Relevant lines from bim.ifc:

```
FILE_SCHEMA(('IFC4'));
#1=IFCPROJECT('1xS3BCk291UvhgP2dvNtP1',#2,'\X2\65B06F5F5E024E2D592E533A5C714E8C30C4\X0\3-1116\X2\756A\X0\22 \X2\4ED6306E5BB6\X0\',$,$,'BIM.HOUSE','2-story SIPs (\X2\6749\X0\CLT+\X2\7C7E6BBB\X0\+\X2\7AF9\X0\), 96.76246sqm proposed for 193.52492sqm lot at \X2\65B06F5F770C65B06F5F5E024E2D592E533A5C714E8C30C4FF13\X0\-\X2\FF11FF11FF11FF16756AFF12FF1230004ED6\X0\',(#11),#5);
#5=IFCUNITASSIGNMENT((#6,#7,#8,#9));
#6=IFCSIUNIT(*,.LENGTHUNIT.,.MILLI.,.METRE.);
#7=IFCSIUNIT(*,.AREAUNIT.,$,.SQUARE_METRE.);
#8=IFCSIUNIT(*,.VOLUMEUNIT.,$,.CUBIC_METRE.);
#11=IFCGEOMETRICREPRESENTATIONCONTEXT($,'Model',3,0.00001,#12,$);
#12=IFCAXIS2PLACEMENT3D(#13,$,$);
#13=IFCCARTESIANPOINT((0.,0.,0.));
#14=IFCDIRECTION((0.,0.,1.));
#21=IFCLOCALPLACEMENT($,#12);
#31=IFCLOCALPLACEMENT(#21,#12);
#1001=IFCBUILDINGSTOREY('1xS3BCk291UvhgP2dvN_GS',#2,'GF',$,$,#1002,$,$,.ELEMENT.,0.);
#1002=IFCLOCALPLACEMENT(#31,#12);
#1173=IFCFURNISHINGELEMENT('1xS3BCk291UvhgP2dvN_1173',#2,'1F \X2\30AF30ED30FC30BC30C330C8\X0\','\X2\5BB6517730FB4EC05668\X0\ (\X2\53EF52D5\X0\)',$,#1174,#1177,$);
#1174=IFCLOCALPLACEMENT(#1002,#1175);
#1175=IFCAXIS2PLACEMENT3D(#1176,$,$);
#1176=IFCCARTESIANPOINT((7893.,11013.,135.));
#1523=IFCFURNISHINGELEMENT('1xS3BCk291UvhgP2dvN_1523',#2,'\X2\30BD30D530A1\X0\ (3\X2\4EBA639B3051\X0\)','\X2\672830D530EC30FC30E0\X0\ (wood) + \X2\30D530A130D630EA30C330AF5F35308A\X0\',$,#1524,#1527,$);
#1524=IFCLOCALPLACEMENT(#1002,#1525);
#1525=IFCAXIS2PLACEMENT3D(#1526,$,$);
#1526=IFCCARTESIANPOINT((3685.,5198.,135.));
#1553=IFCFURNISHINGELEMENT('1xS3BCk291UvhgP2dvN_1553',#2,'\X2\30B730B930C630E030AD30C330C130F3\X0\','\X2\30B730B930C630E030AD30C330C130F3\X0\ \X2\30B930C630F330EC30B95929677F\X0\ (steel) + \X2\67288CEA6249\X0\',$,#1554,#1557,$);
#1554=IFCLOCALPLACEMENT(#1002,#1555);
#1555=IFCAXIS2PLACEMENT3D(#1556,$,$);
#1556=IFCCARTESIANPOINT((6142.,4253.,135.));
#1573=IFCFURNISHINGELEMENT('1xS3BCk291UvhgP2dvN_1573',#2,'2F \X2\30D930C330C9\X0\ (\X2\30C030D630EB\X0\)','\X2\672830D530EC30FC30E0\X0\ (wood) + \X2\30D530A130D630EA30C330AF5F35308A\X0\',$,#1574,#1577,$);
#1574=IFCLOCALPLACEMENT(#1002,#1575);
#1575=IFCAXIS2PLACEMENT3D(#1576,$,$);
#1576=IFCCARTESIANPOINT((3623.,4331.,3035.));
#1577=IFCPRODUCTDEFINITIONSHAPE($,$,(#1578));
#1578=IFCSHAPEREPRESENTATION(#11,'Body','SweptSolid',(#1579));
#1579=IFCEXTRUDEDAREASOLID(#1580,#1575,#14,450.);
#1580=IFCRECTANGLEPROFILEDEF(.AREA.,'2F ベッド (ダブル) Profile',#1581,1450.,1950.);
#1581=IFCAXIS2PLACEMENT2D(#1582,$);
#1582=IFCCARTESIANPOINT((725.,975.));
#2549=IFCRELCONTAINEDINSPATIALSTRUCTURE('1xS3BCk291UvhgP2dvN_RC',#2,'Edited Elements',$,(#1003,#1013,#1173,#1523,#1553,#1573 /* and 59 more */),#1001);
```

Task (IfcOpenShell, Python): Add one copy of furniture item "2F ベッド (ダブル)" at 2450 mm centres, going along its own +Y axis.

```python
import ifcopenshell
import ifcopenshell.api.geometry
import ifcopenshell.api.root
import ifcopenshell.util.element
import ifcopenshell.util.placement

model = ifcopenshell.open("bim.ifc")


def reuse_history(source, copy):
    """copy_class also copies each property set's owner history, people and application; keep the originals."""
    for rel in copy.IsDefinedBy:
        if rel.is_a("IfcRelDefinesByProperties") and (history := rel.RelatingPropertyDefinition.OwnerHistory):
            rel.RelatingPropertyDefinition.OwnerHistory = source.OwnerHistory
            ifcopenshell.util.element.remove_deep2(model, history)


source = model.by_guid("1xS3BCk291UvhgP2dvN_1573")
base = ifcopenshell.util.placement.get_local_placement(source.ObjectPlacement)
step = base[:3, 1] * 2450.0

for i in range(1, 2):
    copy = ifcopenshell.api.root.copy_class(model, product=source)
    copy.Representation = ifcopenshell.util.element.copy_deep(
        model, source.Representation, exclude=["IfcGeometricRepresentationContext", "IfcRepresentationMap"]
    )
    reuse_history(source, copy)
    matrix = base.copy()
    matrix[:3, 3] += i * step
    print("added at", matrix[:3, 3].round(3) + 0.0)
    ifcopenshell.api.geometry.edit_object_placement(model, product=copy, matrix=matrix, is_si=False)

model.write("bim_rev.ifc")
```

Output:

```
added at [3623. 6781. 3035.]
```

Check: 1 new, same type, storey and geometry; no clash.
